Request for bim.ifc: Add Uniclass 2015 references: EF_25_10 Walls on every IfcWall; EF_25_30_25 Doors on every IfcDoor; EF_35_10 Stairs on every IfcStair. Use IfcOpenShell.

First a look at what the model holds.

```python
import ifcopenshell

model = ifcopenshell.open("bim.ifc")
print(model.schema)
print("classifications:", [c.Name for c in model.by_type("IfcClassification")])
for ifc_class in ("IfcDoor", "IfcRoof", "IfcStair", "IfcWall", "IfcWindow"):
    print(ifc_class, len(model.by_type(ifc_class)))
```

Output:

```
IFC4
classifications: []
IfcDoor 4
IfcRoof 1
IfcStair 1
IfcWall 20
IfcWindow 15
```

```python
import ifcopenshell
import ifcopenshell.api.classification

model = ifcopenshell.open("bim.ifc")

system = ifcopenshell.api.classification.add_classification(model, classification="Uniclass 2015")

codes = {
    "IfcWall": ("EF_25_10", "Walls"),
    "IfcDoor": ("EF_25_30_25", "Doors"),
    "IfcStair": ("EF_35_10", "Stairs"),
}
for ifc_class, (code, name) in codes.items():
    products = model.by_type(ifc_class)
    ifcopenshell.api.classification.add_reference(
        model, products=products, classification=system, identification=code, name=name
    )
    print(code, len(products))

model.write("bim_rev.ifc")
```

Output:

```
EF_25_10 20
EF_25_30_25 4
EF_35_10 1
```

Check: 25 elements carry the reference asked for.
